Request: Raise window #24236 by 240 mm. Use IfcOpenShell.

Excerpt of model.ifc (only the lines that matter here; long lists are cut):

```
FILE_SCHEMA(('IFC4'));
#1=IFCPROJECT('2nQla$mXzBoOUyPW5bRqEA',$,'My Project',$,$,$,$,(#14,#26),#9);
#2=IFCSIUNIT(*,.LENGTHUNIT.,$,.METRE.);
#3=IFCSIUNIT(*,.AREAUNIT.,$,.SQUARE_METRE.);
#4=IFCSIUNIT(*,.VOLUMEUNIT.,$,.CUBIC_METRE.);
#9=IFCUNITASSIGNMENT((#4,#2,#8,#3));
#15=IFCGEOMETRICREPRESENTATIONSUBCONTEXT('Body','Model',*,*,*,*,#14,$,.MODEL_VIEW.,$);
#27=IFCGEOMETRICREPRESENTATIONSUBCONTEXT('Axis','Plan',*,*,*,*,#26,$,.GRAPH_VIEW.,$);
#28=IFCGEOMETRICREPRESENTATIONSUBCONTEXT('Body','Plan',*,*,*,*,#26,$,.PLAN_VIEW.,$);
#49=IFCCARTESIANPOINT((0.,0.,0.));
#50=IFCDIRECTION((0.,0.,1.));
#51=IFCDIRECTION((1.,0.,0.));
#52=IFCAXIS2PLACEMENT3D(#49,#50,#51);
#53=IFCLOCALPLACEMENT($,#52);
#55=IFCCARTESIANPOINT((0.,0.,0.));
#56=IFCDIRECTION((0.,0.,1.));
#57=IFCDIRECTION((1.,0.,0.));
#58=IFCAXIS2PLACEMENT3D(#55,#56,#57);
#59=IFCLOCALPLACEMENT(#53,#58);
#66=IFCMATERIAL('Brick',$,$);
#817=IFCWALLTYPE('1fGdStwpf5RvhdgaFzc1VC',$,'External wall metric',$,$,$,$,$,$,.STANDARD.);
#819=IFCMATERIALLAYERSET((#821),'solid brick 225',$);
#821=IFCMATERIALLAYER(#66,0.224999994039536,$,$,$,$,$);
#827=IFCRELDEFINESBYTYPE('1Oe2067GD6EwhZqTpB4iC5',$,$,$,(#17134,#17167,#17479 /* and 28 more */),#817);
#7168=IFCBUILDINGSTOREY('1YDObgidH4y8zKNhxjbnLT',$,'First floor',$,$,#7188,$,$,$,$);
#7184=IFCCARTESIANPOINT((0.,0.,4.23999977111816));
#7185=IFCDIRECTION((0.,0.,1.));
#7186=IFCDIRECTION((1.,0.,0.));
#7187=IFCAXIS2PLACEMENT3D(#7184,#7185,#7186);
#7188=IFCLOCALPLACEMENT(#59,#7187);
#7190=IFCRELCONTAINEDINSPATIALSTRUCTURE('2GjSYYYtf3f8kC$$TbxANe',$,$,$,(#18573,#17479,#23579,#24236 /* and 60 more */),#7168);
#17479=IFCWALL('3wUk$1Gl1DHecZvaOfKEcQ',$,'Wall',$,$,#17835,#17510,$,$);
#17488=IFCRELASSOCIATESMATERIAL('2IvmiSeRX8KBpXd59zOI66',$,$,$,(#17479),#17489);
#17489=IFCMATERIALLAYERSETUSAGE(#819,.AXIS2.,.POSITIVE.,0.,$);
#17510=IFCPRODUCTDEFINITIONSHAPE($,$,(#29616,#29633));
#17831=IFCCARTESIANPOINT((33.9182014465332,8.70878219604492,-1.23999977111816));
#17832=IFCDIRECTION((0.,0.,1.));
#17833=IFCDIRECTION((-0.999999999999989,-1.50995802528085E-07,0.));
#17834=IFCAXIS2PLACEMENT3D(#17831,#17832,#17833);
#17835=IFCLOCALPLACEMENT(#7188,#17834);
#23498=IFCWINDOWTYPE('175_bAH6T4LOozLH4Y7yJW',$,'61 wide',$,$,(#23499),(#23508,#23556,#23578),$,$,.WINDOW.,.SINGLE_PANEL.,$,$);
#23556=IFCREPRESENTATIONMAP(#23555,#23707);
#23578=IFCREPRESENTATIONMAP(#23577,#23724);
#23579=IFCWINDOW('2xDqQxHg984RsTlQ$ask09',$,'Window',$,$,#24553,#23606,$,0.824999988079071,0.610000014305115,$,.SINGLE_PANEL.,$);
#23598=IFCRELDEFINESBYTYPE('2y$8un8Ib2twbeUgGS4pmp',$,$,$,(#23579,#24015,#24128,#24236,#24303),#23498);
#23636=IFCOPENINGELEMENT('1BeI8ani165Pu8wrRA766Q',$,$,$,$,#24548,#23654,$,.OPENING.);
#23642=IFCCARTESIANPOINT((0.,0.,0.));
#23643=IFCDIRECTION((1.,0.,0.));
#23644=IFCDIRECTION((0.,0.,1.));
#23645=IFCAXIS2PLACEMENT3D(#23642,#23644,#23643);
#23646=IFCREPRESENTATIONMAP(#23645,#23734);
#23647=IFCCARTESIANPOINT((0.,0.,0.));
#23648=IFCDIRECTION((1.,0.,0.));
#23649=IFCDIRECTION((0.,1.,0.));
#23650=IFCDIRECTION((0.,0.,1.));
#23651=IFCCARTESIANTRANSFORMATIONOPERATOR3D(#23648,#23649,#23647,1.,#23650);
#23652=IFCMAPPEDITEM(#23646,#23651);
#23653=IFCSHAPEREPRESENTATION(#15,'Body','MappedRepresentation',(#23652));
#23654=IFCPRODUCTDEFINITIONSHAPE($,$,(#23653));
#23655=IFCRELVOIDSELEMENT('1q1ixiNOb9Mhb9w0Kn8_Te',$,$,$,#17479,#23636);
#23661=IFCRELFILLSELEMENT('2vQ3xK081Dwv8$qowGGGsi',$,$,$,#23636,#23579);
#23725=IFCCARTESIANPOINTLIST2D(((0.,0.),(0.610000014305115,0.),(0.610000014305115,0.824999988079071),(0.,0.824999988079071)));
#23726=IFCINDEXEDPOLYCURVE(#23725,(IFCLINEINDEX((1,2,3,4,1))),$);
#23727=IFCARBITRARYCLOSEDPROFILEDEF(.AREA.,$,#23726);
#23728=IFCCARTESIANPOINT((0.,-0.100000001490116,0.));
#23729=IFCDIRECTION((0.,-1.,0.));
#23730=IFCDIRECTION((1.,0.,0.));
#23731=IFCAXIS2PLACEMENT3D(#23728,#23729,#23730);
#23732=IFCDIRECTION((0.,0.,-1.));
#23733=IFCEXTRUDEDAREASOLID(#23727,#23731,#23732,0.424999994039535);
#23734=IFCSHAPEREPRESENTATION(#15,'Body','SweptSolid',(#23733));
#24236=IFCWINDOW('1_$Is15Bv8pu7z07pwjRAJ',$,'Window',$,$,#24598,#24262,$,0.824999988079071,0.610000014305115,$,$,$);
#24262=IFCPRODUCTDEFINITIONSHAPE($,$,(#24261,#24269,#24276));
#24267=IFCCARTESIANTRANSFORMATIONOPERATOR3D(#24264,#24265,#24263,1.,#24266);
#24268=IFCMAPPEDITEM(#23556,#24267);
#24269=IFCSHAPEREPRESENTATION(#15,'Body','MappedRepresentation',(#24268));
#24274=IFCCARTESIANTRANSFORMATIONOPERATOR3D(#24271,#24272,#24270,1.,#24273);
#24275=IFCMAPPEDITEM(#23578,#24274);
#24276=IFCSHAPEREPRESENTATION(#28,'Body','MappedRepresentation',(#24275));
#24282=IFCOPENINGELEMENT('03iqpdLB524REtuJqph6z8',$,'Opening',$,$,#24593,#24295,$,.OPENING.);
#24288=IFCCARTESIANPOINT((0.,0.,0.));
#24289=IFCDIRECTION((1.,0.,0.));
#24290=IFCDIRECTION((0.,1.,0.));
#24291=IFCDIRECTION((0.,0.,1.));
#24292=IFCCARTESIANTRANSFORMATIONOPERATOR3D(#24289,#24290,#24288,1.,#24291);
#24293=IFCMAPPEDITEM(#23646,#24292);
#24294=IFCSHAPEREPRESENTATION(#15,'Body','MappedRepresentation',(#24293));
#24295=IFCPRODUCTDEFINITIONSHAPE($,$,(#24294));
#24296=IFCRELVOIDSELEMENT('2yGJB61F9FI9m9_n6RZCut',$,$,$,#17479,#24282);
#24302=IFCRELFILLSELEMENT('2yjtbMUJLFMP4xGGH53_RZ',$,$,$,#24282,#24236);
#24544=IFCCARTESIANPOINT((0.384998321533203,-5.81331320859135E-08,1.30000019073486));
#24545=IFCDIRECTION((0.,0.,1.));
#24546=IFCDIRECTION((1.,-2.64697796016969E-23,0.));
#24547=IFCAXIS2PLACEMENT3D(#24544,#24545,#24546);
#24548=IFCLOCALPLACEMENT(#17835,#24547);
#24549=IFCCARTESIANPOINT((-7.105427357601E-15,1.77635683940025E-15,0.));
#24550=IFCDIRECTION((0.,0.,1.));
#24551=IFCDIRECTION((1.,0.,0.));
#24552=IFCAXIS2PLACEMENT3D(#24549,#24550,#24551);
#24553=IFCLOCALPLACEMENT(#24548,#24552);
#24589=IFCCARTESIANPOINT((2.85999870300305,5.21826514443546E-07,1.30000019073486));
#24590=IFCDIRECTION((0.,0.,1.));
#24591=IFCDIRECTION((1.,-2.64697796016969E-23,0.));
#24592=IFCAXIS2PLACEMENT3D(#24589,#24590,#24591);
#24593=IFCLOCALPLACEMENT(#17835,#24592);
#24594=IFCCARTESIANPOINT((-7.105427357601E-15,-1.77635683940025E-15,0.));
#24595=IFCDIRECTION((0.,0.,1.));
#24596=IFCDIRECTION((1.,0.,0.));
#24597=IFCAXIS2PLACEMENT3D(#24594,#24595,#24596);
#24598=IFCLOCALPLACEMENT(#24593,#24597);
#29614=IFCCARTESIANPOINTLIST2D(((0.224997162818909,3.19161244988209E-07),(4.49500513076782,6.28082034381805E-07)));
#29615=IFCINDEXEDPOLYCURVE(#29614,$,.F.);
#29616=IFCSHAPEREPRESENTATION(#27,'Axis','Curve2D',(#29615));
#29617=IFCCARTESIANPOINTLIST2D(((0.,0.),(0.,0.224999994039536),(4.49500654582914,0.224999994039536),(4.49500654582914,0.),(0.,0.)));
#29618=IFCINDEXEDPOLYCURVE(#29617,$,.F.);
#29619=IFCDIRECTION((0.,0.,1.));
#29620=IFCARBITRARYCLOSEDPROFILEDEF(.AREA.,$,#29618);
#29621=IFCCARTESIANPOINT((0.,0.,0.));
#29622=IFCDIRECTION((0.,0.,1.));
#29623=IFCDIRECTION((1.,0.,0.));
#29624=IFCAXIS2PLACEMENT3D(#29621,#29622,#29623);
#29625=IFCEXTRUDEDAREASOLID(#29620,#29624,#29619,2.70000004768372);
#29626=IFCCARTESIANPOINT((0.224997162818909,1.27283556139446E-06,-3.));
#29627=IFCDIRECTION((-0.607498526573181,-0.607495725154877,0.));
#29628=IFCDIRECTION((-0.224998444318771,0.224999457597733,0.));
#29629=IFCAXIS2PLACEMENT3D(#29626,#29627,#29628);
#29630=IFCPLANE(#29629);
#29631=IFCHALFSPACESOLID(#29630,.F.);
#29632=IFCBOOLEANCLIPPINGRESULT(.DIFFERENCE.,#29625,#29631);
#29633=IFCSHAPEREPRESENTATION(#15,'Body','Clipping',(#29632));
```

```python
import numpy as np
import ifcopenshell
import ifcopenshell.api.geometry
import ifcopenshell.util.placement
import ifcopenshell.util.unit

model = ifcopenshell.open("model.ifc")
unit_scale = ifcopenshell.util.unit.calculate_unit_scale(model)

window = model.by_guid("1_$Is15Bv8pu7z07pwjRAJ")
opening = window.FillsVoids[0].RelatingOpeningElement
dz = 0.24 / unit_scale

shift = np.array([0.0, 0.0, dz])
# The window is placed relative to its opening, so it follows when the opening moves.
matrix = ifcopenshell.util.placement.get_local_placement(opening.ObjectPlacement)
matrix[:3, 3] += shift
ifcopenshell.api.geometry.edit_object_placement(
    model, product=opening, matrix=matrix, is_si=False, should_transform_children=True
)

print(f"moved by {dz * unit_scale:+.3f} m")

model.write("model_updated.ifc")
```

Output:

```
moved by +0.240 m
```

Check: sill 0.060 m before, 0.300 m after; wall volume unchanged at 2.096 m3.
